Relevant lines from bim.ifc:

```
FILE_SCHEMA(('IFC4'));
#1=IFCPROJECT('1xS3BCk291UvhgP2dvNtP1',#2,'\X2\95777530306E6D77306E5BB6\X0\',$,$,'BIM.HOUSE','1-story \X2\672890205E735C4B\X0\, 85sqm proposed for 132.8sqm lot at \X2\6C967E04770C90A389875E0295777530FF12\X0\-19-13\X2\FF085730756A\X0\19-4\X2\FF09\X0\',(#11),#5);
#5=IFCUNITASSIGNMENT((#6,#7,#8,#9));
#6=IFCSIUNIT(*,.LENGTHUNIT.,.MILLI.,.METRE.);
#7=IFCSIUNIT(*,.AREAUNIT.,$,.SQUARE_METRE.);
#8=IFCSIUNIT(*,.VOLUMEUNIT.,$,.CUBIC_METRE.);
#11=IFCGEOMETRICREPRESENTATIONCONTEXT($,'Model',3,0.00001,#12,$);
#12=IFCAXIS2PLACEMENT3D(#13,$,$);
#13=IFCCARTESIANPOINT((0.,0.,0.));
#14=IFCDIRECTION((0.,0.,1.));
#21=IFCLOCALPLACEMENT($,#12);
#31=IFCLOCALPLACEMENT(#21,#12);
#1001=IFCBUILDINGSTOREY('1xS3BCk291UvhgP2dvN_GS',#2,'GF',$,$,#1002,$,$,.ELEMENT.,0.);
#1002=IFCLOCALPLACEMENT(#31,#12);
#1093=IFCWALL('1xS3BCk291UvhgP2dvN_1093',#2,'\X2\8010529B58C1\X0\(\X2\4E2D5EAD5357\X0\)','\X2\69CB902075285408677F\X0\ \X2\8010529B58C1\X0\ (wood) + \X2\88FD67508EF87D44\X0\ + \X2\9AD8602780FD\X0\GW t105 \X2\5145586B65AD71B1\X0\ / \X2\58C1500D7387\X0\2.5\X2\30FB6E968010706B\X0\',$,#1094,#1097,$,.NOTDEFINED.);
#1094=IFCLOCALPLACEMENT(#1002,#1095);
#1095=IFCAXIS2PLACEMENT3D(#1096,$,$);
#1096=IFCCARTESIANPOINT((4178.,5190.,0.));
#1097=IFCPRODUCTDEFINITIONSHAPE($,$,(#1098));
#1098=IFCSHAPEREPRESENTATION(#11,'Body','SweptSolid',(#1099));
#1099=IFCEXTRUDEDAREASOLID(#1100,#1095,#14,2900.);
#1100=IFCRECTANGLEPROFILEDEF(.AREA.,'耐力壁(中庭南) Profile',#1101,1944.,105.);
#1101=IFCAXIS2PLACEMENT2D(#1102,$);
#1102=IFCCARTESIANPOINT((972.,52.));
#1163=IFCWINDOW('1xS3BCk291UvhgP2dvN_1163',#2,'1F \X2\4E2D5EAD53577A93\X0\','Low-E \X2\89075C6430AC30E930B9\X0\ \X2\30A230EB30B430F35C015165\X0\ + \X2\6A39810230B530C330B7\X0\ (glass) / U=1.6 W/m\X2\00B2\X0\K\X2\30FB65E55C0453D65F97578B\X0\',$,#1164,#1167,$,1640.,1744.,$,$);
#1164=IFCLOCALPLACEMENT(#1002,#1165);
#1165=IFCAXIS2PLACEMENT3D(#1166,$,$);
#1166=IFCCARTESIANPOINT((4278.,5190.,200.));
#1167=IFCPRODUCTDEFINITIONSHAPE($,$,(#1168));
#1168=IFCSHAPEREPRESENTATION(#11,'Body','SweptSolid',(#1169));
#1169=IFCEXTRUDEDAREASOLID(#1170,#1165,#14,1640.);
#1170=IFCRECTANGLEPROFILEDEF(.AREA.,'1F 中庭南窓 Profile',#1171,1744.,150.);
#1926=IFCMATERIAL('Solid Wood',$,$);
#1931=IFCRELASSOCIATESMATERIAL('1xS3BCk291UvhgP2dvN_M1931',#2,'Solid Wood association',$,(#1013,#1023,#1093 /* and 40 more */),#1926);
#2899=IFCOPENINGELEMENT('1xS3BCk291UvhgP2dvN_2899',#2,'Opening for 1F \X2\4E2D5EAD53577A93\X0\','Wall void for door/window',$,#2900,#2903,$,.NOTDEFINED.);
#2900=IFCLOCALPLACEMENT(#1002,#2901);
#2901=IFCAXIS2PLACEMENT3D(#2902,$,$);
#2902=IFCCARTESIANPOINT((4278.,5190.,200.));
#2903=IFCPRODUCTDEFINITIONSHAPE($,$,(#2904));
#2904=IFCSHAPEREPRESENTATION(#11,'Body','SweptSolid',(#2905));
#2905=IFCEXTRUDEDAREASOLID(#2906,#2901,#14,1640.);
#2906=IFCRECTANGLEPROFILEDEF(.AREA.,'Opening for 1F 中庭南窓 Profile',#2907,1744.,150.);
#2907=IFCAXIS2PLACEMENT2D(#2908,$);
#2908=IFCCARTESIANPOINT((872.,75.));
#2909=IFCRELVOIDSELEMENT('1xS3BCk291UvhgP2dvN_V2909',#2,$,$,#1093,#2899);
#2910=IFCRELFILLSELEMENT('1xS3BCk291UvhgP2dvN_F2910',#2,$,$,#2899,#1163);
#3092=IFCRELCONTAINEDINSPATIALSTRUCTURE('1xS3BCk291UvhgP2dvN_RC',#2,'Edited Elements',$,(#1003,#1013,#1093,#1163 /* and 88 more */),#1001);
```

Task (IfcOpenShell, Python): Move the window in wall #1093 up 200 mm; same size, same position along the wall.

```python
import numpy as np
import ifcopenshell
import ifcopenshell.api.geometry
import ifcopenshell.util.placement
import ifcopenshell.util.unit

model = ifcopenshell.open("bim.ifc")
unit_scale = ifcopenshell.util.unit.calculate_unit_scale(model)

window = model.by_id(1163)
opening = window.FillsVoids[0].RelatingOpeningElement
dz = 0.2 / unit_scale

shift = np.array([0.0, 0.0, dz])
# The window is not placed relative to its opening, so move both.
for product in (opening, window):
    matrix = ifcopenshell.util.placement.get_local_placement(product.ObjectPlacement)
    matrix[:3, 3] += shift
    ifcopenshell.api.geometry.edit_object_placement(model, product=product, matrix=matrix, is_si=False)

print(f"moved by {dz * unit_scale:+.3f} m")

model.write("bim_rev.ifc")
```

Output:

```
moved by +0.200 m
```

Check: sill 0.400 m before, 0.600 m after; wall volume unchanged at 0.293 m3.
